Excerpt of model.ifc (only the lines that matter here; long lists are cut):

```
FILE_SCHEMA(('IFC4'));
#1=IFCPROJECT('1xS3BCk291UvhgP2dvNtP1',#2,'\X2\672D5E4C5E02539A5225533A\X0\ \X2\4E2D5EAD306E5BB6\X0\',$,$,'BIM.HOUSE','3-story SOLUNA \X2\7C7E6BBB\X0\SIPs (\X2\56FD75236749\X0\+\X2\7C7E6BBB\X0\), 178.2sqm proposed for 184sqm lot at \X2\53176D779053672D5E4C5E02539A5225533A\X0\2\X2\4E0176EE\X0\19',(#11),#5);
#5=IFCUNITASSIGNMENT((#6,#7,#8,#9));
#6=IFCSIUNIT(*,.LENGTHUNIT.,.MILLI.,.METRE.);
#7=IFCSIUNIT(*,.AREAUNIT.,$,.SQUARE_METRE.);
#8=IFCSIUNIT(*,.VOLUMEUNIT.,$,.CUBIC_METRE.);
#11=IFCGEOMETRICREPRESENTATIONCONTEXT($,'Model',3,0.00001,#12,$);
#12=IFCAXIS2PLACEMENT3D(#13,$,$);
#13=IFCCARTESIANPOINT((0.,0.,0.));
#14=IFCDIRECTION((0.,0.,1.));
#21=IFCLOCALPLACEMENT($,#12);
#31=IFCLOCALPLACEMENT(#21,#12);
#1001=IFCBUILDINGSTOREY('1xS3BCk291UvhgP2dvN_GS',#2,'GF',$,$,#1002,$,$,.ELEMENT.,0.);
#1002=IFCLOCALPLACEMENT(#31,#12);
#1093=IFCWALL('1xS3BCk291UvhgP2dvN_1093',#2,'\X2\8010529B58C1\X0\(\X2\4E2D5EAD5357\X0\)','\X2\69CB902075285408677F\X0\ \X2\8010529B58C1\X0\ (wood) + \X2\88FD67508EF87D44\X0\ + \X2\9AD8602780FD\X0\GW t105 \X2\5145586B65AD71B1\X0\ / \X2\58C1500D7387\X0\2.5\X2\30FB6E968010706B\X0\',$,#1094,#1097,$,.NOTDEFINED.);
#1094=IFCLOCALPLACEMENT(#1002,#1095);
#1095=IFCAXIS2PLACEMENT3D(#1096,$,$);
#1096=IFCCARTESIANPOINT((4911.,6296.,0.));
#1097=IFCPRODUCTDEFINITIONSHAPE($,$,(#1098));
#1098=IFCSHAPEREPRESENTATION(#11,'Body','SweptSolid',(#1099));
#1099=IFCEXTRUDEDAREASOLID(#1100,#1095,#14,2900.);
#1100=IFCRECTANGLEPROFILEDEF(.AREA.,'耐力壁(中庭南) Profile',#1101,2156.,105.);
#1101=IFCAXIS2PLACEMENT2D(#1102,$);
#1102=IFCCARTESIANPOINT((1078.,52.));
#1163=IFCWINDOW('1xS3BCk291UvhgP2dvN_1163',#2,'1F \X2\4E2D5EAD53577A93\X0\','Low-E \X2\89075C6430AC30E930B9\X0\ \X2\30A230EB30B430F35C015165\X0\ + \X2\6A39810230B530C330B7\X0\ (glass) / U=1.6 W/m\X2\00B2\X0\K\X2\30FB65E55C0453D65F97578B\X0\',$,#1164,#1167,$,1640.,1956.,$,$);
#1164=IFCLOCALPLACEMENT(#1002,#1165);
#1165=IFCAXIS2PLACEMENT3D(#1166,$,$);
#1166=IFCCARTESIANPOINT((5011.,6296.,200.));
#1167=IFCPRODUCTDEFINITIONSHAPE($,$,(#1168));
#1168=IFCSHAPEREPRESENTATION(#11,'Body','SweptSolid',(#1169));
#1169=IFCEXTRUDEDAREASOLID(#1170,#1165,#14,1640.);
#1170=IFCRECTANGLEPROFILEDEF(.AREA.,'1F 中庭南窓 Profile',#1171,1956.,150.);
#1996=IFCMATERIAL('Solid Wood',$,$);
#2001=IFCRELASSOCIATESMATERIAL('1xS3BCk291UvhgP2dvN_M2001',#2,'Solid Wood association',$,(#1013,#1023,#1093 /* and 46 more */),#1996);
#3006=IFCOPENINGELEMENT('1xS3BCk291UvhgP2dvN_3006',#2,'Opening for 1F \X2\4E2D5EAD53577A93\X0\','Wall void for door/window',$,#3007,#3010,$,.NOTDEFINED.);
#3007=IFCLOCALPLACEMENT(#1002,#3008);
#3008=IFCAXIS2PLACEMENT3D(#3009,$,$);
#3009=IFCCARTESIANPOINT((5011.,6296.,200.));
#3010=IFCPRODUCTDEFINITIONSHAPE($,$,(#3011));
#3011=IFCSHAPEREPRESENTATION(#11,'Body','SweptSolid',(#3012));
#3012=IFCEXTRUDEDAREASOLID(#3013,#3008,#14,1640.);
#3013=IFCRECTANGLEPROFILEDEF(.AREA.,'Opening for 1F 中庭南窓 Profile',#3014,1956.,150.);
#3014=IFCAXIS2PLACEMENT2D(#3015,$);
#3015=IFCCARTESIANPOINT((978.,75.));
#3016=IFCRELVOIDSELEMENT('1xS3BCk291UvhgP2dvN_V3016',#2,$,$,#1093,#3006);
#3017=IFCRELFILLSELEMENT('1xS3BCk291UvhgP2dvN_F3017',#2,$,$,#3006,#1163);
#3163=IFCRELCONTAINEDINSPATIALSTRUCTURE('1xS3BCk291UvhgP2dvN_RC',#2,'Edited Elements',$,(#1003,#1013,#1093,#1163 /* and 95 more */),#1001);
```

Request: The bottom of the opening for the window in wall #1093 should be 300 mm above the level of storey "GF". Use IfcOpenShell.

```python
import numpy as np
import ifcopenshell
import ifcopenshell.api.geometry
import ifcopenshell.geom
import ifcopenshell.util.element
import ifcopenshell.util.placement
import ifcopenshell.util.shape
import ifcopenshell.util.unit

model = ifcopenshell.open("model.ifc")
unit_scale = ifcopenshell.util.unit.calculate_unit_scale(model)

window = model.by_guid("1xS3BCk291UvhgP2dvN_1163")
opening = window.FillsVoids[0].RelatingOpeningElement
storey = ifcopenshell.util.element.get_container(window, ifc_class="IfcBuildingStorey")
level = ifcopenshell.util.placement.get_local_placement(storey.ObjectPlacement)[2, 3]

# The opening's origin need not be at the sill, so measure its lowest point.
shape = ifcopenshell.geom.create_shape(ifcopenshell.geom.settings(), opening)
bottom = ifcopenshell.util.shape.get_shape_bottom_elevation(shape, shape.geometry) / unit_scale
dz = level + 300.0 - bottom

shift = np.array([0.0, 0.0, dz])
# The window is not placed relative to its opening, so move both.
for product in (opening, window):
    matrix = ifcopenshell.util.placement.get_local_placement(product.ObjectPlacement)
    matrix[:3, 3] += shift
    ifcopenshell.api.geometry.edit_object_placement(model, product=product, matrix=matrix, is_si=False)

print(f"moved by {dz * unit_scale:+.3f} m")

model.write("model_edited.ifc")
```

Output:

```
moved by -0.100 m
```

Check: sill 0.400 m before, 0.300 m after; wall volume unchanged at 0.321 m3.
